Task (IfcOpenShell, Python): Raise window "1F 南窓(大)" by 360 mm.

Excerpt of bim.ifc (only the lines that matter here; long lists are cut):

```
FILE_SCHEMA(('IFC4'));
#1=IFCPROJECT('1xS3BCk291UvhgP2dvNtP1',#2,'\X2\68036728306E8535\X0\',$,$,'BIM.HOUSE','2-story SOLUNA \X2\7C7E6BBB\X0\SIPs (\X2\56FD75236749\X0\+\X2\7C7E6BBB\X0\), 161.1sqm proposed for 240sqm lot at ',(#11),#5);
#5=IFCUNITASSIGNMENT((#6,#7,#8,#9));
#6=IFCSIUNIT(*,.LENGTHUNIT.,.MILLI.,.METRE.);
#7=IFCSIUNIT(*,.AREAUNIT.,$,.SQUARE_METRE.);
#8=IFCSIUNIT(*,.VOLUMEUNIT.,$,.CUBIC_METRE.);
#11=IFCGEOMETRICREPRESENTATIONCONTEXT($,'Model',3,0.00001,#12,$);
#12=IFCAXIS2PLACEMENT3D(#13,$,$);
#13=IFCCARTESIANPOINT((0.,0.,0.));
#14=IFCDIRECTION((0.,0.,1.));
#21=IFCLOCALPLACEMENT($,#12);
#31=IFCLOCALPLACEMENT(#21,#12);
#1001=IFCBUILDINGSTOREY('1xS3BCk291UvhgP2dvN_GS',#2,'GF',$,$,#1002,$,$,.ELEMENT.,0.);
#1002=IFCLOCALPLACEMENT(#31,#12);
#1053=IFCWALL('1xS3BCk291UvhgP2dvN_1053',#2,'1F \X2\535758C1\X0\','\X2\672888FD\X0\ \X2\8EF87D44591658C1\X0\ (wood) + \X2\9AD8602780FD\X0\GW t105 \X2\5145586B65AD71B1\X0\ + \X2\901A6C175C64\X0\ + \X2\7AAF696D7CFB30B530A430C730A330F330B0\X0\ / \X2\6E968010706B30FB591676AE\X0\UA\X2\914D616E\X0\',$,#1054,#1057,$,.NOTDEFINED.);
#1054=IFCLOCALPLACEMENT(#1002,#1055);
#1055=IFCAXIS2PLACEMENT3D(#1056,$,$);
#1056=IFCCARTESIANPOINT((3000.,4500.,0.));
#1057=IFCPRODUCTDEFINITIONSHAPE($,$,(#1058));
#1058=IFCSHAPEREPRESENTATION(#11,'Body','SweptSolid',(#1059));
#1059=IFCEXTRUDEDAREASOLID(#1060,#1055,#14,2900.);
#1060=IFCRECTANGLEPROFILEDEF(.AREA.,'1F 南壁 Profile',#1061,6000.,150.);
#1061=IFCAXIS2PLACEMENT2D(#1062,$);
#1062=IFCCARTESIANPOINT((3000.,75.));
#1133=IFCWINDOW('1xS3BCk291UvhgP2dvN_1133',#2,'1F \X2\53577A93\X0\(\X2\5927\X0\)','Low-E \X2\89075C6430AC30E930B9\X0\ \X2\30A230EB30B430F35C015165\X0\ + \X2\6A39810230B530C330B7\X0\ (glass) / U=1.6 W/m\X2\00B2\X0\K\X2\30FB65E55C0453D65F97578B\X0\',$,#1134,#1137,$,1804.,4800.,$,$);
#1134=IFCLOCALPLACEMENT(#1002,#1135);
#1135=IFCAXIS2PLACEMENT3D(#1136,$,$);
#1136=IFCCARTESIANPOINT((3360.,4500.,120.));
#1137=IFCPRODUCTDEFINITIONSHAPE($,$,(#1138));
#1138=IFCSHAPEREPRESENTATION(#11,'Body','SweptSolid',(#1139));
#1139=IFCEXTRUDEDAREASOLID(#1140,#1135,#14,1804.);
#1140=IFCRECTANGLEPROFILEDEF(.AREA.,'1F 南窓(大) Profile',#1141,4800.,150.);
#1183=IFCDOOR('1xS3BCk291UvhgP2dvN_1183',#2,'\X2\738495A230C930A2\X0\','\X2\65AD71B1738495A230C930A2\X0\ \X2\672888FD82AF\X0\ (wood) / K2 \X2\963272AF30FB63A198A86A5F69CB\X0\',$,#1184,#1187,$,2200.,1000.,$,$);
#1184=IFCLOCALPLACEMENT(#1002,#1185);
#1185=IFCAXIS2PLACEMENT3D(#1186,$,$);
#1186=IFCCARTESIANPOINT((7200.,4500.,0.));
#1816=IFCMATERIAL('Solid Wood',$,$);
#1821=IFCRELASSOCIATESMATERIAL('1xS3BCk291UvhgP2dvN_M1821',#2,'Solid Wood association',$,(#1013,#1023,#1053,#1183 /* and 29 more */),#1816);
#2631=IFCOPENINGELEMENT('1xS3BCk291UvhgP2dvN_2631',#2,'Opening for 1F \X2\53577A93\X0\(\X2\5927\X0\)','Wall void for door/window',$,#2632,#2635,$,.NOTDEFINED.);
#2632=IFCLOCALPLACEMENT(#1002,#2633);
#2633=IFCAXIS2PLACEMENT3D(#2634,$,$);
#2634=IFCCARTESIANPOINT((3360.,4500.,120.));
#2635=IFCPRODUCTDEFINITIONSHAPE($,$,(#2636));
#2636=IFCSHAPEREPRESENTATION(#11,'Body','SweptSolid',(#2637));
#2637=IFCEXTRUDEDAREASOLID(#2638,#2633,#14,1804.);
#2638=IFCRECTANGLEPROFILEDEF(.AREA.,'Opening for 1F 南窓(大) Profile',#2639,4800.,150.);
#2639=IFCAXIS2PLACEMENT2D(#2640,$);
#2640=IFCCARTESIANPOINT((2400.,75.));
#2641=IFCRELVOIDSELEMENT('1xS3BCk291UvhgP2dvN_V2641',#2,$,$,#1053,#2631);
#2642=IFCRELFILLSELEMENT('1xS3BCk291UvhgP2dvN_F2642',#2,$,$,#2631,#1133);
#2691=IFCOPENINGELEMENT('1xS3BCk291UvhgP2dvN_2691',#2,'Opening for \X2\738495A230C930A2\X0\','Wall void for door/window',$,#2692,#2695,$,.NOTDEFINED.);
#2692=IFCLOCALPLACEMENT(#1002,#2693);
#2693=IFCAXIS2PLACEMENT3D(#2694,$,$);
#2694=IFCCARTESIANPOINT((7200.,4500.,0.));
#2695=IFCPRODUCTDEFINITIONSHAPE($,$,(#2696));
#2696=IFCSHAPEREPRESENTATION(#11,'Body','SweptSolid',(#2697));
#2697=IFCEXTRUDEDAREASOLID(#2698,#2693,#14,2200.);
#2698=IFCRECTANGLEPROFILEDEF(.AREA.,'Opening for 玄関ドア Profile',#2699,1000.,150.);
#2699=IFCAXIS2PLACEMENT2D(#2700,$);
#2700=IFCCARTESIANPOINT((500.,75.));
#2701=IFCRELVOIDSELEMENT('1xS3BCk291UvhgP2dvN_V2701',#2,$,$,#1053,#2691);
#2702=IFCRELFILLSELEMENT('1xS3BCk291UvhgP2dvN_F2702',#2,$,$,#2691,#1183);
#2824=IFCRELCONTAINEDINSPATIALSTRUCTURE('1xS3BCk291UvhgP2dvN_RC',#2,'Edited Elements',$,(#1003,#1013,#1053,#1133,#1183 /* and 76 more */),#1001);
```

```python
import numpy as np
import ifcopenshell
import ifcopenshell.api.geometry
import ifcopenshell.util.placement
import ifcopenshell.util.unit

model = ifcopenshell.open("bim.ifc")
unit_scale = ifcopenshell.util.unit.calculate_unit_scale(model)

window = model.by_id(1133)
opening = window.FillsVoids[0].RelatingOpeningElement
dz = 360.0

shift = np.array([0.0, 0.0, dz])
# The window is not placed relative to its opening, so move both.
for product in (opening, window):
    matrix = ifcopenshell.util.placement.get_local_placement(product.ObjectPlacement)
    matrix[:3, 3] += shift
    ifcopenshell.api.geometry.edit_object_placement(model, product=product, matrix=matrix, is_si=False)

print(f"moved by {dz * unit_scale:+.3f} m")

model.write("bim_updated.ifc")
```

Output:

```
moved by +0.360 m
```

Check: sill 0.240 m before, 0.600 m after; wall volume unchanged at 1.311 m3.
